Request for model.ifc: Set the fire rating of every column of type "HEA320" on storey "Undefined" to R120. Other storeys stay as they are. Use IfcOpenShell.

First a look at what the model holds.

```python
import ifcopenshell
import ifcopenshell.util.element

model = ifcopenshell.open("model.ifc")
print(model.schema)
storey = next(s for s in model.by_type("IfcBuildingStorey") if s.Name == "Undefined")
columns = [e for e in ifcopenshell.util.element.get_decomposition(storey) if e.is_a("IfcColumn")]
seen = {}
for e in columns:
    element_type = ifcopenshell.util.element.get_type(e)
    key = (element_type.Name if element_type != e and element_type else None, ifcopenshell.util.element.get_pset(e, "Pset_ColumnCommon", "FireRating"))
    seen[key] = seen.get(key, 0) + 1
for (name, value), count in sorted(seen.items(), key=str):
    print(count, "x", name, "|", value)
```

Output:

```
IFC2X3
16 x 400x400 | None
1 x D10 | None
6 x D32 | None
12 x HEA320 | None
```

```python
import ifcopenshell
import ifcopenshell.api.pset
import ifcopenshell.util.element

model = ifcopenshell.open("model.ifc")

storey = next(s for s in model.by_type("IfcBuildingStorey") if s.Name == "Undefined")
columns = [e for e in ifcopenshell.util.element.get_decomposition(storey) if e.is_a("IfcColumn")]

count = 0
for e in columns:
    element_type = ifcopenshell.util.element.get_type(e)
    if element_type in (None, e) or element_type.Name != "HEA320":
        continue
    found = ifcopenshell.util.element.get_pset(e, "Pset_ColumnCommon", should_inherit=False)
    if found:
        pset = model.by_id(found["id"])
        if len(ifcopenshell.util.element.get_elements_by_pset(pset)) > 1:
            pset = ifcopenshell.api.pset.unshare_pset(model, products=[e], pset=pset)[0]
    else:
        pset = ifcopenshell.api.pset.add_pset(model, product=e, name="Pset_ColumnCommon")
    ifcopenshell.api.pset.edit_pset(model, pset=pset, properties={"FireRating": "R120"})
    count += 1

print(count, "columns updated")

model.write("model_edited.ifc")
```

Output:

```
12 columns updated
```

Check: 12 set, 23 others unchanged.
